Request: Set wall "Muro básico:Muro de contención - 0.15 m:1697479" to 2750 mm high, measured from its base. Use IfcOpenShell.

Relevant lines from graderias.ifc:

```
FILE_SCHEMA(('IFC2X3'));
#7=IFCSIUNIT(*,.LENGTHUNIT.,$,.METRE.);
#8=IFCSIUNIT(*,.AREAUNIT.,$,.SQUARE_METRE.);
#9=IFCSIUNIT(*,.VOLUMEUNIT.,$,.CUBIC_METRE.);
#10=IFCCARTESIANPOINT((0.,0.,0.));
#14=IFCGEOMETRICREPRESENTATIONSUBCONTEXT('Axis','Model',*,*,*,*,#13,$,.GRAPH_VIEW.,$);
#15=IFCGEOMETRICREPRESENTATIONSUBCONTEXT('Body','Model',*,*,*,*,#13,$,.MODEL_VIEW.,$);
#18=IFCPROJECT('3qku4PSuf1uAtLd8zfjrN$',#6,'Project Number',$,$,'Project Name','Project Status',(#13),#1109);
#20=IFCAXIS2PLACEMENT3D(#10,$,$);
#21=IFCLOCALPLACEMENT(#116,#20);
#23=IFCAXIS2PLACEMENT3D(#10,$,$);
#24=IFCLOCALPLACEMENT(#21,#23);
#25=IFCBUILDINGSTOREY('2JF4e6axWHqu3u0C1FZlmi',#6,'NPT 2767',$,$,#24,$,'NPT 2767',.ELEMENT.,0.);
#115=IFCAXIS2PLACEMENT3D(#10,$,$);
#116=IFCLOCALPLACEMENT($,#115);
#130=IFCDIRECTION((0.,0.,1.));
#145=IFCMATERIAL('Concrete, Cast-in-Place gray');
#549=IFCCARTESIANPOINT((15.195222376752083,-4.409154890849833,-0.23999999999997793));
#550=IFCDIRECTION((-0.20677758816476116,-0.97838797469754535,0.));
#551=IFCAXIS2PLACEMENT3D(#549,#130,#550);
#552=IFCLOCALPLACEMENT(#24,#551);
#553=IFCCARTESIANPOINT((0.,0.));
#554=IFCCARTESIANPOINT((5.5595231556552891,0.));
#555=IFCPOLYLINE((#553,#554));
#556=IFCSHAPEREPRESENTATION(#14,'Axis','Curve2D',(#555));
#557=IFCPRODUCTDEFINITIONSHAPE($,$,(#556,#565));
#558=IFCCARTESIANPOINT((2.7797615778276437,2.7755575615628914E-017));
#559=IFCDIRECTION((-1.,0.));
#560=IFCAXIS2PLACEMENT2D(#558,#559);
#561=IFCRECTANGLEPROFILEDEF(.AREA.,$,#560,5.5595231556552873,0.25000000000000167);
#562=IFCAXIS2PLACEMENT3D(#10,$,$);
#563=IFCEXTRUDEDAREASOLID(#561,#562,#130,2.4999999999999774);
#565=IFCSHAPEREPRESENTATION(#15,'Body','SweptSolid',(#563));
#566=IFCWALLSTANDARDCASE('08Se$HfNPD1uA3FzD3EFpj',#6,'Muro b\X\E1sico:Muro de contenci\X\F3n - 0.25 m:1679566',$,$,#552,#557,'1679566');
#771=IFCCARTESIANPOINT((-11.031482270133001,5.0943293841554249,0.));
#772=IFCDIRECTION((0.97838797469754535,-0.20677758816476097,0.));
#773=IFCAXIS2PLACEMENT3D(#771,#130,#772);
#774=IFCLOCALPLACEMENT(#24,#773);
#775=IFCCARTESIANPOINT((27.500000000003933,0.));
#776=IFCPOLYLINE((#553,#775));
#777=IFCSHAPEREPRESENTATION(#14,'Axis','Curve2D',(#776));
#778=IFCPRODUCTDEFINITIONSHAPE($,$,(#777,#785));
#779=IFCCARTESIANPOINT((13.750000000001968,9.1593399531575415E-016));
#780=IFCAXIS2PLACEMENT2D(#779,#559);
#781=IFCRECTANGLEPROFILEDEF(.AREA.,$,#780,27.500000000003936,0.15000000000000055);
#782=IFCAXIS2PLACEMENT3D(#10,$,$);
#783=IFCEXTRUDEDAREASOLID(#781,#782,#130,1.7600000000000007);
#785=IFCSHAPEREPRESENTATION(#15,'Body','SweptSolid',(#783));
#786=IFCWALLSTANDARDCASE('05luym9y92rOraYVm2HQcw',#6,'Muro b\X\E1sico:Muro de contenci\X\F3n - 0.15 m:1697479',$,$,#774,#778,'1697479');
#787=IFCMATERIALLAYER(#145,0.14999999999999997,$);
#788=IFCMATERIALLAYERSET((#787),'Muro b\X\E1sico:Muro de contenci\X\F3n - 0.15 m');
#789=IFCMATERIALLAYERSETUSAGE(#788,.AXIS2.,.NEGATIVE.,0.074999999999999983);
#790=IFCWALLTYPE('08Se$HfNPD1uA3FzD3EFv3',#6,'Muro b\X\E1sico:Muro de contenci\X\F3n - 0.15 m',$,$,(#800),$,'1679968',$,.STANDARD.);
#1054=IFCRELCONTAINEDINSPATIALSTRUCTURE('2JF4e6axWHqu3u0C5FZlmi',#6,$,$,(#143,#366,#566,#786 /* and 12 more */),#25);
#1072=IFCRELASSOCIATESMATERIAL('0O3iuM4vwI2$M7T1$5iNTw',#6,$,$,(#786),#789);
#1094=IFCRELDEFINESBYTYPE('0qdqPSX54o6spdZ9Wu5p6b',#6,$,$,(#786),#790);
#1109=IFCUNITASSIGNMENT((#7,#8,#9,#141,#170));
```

```python
import ifcopenshell
import ifcopenshell.geom
import ifcopenshell.util.representation
import ifcopenshell.util.shape
import ifcopenshell.util.unit

model = ifcopenshell.open("graderias.ifc")
unit_scale = ifcopenshell.util.unit.calculate_unit_scale(model)
settings = ifcopenshell.geom.settings()


def volume(element):
    """Net volume in cubic metres, openings subtracted."""
    shape = ifcopenshell.geom.create_shape(settings, element)
    return ifcopenshell.util.shape.get_volume(shape.geometry)


wall = model.by_guid("05luym9y92rOraYVm2HQcw")
before = volume(wall)

body = ifcopenshell.util.representation.get_representation(wall, "Model", "Body")
solid = body.Items[0]
old_height = solid.Depth
solid.Depth = 2.75 / unit_scale
after = volume(wall)

print(f"height {old_height:g} -> {solid.Depth:g}, volume {before:.3f} -> {after:.3f} m3")

model.write("graderias_updated.ifc")
```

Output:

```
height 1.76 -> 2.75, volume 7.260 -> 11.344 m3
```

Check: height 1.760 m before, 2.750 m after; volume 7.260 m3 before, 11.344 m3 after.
